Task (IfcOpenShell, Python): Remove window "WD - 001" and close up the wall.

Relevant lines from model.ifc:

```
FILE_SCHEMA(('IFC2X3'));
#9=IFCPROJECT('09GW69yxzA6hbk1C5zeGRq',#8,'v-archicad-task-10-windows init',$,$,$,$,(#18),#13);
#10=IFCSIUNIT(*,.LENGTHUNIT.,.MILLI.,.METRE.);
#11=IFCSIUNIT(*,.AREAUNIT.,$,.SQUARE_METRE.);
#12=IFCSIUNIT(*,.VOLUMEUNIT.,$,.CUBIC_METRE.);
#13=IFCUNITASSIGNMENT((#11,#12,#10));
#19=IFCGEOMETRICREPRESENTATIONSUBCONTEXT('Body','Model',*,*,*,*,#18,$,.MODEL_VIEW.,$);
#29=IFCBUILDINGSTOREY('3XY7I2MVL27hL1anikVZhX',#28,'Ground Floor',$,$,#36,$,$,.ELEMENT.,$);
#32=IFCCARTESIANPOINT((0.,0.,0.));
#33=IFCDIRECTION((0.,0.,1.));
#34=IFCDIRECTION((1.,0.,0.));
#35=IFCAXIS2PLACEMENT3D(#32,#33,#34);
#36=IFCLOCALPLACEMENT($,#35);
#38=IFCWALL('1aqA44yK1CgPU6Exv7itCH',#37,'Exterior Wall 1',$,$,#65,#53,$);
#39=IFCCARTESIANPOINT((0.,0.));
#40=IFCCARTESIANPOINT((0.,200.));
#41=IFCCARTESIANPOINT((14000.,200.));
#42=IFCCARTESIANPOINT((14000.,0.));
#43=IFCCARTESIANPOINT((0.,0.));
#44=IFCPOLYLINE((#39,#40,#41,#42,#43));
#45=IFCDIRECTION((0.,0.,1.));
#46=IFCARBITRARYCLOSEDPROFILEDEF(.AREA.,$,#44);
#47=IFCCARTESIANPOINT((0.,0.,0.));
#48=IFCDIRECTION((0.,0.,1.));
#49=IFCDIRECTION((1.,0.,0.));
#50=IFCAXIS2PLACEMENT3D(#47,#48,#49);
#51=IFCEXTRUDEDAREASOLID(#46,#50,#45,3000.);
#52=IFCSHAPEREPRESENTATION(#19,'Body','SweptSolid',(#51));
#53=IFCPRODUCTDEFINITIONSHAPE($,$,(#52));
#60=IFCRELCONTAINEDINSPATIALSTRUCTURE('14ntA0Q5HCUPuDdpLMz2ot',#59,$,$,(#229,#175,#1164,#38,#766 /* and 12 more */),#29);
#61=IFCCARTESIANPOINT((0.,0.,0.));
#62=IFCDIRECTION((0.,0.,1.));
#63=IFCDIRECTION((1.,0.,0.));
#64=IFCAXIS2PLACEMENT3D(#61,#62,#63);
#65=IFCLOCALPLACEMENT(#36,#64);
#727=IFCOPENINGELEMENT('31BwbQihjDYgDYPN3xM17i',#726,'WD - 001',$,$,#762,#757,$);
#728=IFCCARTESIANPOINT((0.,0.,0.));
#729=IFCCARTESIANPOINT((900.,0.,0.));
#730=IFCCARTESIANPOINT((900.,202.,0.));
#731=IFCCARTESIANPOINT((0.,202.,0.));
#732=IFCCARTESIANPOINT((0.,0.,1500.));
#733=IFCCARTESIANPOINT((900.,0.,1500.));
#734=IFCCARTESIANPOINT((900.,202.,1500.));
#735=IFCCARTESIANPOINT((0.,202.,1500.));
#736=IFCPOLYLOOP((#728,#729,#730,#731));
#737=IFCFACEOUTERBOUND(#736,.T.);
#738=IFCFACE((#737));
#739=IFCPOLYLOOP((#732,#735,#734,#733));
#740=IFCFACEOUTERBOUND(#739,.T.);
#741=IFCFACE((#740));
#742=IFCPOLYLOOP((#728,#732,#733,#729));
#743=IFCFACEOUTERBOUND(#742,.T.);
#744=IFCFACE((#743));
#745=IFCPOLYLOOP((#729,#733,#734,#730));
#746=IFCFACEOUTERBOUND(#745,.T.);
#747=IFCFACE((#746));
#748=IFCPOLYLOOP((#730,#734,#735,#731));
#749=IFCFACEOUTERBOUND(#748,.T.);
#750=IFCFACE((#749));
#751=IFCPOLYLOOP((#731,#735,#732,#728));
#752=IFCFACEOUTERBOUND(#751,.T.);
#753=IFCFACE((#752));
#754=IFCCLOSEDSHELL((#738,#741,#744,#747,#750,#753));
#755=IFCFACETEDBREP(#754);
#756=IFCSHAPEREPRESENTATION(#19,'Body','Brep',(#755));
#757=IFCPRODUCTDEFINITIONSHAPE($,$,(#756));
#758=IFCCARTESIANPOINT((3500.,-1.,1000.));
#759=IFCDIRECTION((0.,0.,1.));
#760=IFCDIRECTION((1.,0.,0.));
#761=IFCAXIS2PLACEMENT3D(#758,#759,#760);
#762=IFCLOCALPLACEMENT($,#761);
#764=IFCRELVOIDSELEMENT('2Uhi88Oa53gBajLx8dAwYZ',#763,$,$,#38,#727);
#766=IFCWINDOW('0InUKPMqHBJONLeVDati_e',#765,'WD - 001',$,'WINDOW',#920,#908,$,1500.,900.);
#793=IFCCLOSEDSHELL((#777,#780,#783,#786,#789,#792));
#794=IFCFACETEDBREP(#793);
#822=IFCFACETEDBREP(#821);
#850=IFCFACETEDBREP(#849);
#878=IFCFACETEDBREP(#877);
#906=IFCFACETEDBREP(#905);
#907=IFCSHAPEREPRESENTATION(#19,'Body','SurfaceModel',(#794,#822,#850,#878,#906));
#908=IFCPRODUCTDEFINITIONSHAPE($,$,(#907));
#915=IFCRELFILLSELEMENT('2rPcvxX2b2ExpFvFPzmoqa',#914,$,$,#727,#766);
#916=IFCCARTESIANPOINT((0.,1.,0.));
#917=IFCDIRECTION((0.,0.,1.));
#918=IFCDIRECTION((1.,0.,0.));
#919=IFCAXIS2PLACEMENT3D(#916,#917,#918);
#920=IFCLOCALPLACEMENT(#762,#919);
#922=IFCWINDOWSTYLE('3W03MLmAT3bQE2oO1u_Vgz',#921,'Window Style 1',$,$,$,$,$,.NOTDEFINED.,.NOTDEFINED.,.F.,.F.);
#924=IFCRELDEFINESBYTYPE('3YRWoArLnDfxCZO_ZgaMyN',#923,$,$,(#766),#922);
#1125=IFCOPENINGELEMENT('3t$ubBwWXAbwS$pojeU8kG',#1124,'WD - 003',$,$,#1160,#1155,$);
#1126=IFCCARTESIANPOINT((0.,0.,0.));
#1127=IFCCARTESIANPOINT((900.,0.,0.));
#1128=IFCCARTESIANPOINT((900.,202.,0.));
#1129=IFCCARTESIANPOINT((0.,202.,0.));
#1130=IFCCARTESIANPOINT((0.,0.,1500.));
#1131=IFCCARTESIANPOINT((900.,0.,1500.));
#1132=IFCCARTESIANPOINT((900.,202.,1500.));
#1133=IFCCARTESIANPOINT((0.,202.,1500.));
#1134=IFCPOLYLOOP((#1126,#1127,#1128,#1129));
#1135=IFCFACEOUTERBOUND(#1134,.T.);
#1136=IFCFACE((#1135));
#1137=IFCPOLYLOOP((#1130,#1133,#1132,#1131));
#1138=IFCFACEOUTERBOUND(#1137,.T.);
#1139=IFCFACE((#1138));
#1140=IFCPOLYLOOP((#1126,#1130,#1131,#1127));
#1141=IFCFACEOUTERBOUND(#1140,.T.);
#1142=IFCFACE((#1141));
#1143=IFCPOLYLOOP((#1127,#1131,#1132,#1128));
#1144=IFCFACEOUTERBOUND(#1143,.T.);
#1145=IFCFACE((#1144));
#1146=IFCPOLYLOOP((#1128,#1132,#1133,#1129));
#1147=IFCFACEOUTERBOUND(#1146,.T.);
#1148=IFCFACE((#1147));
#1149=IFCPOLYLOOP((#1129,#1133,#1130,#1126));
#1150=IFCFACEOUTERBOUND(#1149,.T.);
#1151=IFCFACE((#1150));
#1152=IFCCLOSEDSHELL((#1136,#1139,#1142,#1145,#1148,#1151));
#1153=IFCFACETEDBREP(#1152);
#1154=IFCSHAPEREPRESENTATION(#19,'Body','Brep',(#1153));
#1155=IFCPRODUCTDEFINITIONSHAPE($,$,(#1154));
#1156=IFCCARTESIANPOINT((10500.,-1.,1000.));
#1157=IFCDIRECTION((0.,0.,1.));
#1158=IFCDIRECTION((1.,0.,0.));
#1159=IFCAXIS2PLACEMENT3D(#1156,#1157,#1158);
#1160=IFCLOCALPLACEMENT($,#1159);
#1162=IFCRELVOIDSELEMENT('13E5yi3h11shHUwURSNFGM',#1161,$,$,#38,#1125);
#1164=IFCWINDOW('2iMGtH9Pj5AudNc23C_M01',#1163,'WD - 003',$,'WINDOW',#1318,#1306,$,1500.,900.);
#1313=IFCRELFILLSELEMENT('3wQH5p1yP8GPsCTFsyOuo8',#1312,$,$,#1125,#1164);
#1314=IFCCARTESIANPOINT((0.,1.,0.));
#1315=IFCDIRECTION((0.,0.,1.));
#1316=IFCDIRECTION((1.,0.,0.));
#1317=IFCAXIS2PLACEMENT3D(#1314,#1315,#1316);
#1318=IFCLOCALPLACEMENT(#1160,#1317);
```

```python
import ifcopenshell
import ifcopenshell.api.feature
import ifcopenshell.api.root
import ifcopenshell.geom
import ifcopenshell.util.shape

model = ifcopenshell.open("model.ifc")
settings = ifcopenshell.geom.settings()


def volume(element):
    """Net volume in cubic metres, openings subtracted."""
    shape = ifcopenshell.geom.create_shape(settings, element)
    return ifcopenshell.util.shape.get_volume(shape.geometry)


window = model.by_guid("0InUKPMqHBJONLeVDati_e")
opening = window.FillsVoids[0].RelatingOpeningElement
wall = opening.VoidsElements[0].RelatingBuildingElement
before = volume(wall)

ifcopenshell.api.root.remove_product(model, product=window)
ifcopenshell.api.feature.remove_feature(model, feature=opening)

after = volume(wall)

print(f"wall volume {before:.3f} -> {after:.3f} m3")

model.write("model_v2.ifc")
```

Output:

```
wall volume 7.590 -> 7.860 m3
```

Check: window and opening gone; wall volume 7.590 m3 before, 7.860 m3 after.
